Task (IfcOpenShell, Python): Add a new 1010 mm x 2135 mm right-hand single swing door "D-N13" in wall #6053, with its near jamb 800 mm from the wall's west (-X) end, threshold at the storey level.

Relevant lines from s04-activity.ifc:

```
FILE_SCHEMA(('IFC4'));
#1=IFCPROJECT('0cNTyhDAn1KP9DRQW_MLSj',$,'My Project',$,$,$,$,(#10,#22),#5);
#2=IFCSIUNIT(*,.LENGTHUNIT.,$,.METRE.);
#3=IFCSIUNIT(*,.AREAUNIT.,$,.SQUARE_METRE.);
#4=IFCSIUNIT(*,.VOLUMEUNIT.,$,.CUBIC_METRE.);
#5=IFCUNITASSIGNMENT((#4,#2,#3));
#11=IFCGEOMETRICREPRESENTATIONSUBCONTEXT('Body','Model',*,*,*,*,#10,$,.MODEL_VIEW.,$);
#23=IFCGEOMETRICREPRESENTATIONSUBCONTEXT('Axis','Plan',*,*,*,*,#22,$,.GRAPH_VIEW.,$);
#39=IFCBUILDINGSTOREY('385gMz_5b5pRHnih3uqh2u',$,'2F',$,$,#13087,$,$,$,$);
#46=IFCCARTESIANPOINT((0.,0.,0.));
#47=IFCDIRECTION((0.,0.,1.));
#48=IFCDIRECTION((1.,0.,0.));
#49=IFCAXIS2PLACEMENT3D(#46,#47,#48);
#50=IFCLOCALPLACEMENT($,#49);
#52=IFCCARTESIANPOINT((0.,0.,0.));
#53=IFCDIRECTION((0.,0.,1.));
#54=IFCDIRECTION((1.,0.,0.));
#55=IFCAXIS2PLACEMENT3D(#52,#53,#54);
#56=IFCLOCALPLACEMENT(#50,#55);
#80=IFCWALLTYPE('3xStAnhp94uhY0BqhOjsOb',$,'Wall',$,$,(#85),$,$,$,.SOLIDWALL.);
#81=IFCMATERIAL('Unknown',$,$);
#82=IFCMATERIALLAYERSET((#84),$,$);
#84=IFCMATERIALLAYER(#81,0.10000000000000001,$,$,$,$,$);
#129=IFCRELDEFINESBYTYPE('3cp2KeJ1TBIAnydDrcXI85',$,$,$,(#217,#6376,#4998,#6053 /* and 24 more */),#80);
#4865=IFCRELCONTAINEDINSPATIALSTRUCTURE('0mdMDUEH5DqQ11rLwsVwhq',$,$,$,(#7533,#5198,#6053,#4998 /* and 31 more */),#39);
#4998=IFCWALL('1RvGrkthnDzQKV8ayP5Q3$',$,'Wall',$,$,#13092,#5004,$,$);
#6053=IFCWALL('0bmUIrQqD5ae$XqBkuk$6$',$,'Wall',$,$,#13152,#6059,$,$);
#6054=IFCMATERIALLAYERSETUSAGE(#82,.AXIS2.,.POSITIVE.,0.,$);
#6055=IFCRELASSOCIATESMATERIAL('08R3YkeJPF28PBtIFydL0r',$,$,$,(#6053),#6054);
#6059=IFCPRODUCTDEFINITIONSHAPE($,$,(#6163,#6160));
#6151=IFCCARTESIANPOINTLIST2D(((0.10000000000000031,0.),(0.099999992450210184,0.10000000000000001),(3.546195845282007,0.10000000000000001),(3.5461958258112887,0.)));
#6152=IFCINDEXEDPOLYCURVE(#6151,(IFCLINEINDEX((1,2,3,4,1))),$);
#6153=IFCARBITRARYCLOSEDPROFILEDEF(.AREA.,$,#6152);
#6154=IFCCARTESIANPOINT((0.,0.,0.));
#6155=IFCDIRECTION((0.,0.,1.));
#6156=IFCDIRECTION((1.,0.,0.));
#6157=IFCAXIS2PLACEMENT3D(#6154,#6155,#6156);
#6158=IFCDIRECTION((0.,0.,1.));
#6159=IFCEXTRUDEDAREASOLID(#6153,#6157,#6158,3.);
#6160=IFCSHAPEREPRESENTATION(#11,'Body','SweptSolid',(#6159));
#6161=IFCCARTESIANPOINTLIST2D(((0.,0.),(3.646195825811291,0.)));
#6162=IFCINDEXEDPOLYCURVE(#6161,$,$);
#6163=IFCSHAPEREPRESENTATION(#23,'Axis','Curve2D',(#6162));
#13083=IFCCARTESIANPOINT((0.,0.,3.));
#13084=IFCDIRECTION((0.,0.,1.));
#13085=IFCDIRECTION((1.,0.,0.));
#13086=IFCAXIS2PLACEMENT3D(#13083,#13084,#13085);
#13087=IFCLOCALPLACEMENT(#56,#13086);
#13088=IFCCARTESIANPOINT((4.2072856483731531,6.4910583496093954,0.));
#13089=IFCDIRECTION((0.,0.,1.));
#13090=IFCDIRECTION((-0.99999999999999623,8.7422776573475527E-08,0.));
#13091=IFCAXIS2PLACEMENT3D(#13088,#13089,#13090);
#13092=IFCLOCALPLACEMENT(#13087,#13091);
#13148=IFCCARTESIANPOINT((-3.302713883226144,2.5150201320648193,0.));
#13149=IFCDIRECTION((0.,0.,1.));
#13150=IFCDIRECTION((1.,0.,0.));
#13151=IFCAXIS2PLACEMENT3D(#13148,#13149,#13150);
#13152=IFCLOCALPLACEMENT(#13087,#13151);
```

```python
import numpy as np
import ifcopenshell
import ifcopenshell.api.feature
import ifcopenshell.api.geometry
import ifcopenshell.api.root
import ifcopenshell.api.spatial
import ifcopenshell.geom
import ifcopenshell.util.element
import ifcopenshell.util.placement
import ifcopenshell.util.representation
import ifcopenshell.util.shape
import ifcopenshell.util.unit

model = ifcopenshell.open("s04-activity.ifc")
unit_scale = ifcopenshell.util.unit.calculate_unit_scale(model)
settings = ifcopenshell.geom.settings()


def volume(element):
    """Net volume in cubic metres, openings subtracted."""
    shape = ifcopenshell.geom.create_shape(settings, element)
    return ifcopenshell.util.shape.get_volume(shape.geometry)


wall = model.by_guid("0bmUIrQqD5ae$XqBkuk$6$")
storey = ifcopenshell.util.element.get_container(wall, ifc_class="IfcBuildingStorey")
context = ifcopenshell.util.representation.get_context(model, "Model", "Body", "MODEL_VIEW")
before = volume(wall)

width, height, from_end, sill = 1.01, 2.135, 0.8, 0.0  # metres

# The wall runs along its own X axis, and the end named is its -X end.
wall_shape = ifcopenshell.geom.create_shape(settings, wall)
x, y, z = ifcopenshell.util.shape.get_vertices(wall_shape.geometry).T
start = x.min() + from_end
face, thickness = float(y.min()), float(y.max() - y.min())
wall_matrix = ifcopenshell.util.placement.get_local_placement(wall.ObjectPlacement)
level = ifcopenshell.util.placement.get_local_placement(storey.ObjectPlacement)[2, 3]


def in_wall(x, y):
    """Placement at x, y metres in the wall's axes, at sill height."""
    matrix = wall_matrix.copy()
    matrix[:, 3] = wall_matrix @ np.array([x / unit_scale, y / unit_scale, 0.0, 1.0])
    matrix[2, 3] = level + sill / unit_scale
    return matrix


# Opening: a box that overshoots both wall faces by 50 mm.
opening = ifcopenshell.api.root.create_entity(model, ifc_class="IfcOpeningElement", predefined_type="OPENING")
box = ifcopenshell.api.geometry.add_wall_representation(
    model, context=context, length=width, height=height, thickness=thickness + 0.1
)
ifcopenshell.api.geometry.assign_representation(model, product=opening, representation=box)
ifcopenshell.api.geometry.edit_object_placement(model, product=opening, matrix=in_wall(start, face - 0.05), is_si=False)
ifcopenshell.api.feature.add_feature(model, feature=opening, element=wall)

door = ifcopenshell.api.root.create_entity(model, ifc_class="IfcDoor", name="D-N13", predefined_type="DOOR")
door.OverallWidth, door.OverallHeight = width / unit_scale, height / unit_scale
door.OperationType = "SINGLE_SWING_RIGHT"
body = ifcopenshell.api.geometry.add_door_representation(
    model,
    context=context,
    overall_width=door.OverallWidth,
    overall_height=door.OverallHeight,
    operation_type="SINGLE_SWING_RIGHT",
    lining_properties={"LiningDepth": thickness / unit_scale, "ThresholdDepth": thickness / unit_scale},
)
ifcopenshell.api.geometry.assign_representation(model, product=door, representation=body)
ifcopenshell.api.spatial.assign_container(model, products=[door], relating_structure=storey)
ifcopenshell.api.feature.add_filling(model, opening=opening, element=door)

# The lining spans the wall, so the door starts at the wall face.
ifcopenshell.api.geometry.edit_object_placement(model, product=door, matrix=in_wall(start, face), is_si=False)

after = volume(wall)

print(f"wall volume {before:.3f} -> {after:.3f} m3")

model.write("s04-activity_rev.ifc")
```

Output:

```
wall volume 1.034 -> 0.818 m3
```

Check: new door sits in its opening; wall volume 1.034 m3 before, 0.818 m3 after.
